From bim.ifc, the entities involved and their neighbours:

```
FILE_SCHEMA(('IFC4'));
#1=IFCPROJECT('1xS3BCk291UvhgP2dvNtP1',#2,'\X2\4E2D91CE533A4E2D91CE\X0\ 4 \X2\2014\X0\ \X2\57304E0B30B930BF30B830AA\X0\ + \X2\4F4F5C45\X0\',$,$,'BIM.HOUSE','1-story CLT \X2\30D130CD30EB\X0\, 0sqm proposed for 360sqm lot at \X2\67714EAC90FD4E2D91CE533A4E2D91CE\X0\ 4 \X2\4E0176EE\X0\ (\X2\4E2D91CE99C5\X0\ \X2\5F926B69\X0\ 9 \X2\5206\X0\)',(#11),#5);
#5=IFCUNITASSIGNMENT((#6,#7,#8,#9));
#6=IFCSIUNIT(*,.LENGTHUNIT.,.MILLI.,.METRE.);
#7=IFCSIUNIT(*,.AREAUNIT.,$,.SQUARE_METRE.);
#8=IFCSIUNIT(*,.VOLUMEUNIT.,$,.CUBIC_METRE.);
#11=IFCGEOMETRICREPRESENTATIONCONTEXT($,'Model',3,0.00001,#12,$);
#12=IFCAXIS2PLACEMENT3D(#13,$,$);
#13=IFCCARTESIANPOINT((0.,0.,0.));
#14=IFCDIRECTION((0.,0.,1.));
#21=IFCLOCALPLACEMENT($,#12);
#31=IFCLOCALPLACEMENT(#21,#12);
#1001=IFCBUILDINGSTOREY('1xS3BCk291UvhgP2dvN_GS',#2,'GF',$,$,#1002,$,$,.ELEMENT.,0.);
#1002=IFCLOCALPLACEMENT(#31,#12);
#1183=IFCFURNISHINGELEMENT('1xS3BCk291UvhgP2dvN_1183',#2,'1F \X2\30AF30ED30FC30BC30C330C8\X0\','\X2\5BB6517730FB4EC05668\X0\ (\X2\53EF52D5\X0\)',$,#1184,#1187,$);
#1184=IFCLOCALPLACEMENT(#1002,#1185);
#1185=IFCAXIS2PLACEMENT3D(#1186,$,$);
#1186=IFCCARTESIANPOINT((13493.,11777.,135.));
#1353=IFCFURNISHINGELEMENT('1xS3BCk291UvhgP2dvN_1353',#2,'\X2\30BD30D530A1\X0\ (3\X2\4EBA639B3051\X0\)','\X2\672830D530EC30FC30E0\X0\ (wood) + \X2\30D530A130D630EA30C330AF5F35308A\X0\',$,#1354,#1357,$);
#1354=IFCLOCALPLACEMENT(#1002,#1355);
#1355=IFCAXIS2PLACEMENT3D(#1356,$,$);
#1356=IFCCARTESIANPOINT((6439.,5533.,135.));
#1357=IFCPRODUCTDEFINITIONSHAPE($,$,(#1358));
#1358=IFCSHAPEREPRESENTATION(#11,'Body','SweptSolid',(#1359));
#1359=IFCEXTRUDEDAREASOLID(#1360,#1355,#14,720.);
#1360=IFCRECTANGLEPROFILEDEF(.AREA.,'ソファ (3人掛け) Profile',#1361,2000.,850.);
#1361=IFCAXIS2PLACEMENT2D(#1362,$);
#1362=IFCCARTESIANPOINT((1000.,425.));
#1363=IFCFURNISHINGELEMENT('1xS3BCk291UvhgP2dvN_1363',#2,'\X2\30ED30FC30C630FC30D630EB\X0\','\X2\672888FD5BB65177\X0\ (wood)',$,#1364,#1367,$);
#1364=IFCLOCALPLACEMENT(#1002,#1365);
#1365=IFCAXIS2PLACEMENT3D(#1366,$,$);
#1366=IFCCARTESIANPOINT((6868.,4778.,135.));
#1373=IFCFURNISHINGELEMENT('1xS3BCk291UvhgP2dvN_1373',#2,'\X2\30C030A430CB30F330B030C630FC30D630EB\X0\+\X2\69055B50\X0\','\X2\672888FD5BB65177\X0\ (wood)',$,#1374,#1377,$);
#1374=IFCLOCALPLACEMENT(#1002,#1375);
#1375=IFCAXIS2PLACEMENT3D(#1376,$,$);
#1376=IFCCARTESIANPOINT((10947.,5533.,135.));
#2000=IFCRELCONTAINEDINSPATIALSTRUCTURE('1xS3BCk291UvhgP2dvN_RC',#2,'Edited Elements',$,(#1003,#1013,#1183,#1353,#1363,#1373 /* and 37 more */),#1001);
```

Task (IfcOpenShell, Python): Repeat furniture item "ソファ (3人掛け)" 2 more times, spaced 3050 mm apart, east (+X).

```python
import numpy as np
import ifcopenshell
import ifcopenshell.api.geometry
import ifcopenshell.api.root
import ifcopenshell.util.element
import ifcopenshell.util.placement
import ifcopenshell.util.unit

model = ifcopenshell.open("bim.ifc")
unit_scale = ifcopenshell.util.unit.calculate_unit_scale(model)


def reuse_history(source, copy):
    """copy_class also copies each property set's owner history, people and application; keep the originals."""
    for rel in copy.IsDefinedBy:
        if rel.is_a("IfcRelDefinesByProperties") and (history := rel.RelatingPropertyDefinition.OwnerHistory):
            rel.RelatingPropertyDefinition.OwnerHistory = source.OwnerHistory
            ifcopenshell.util.element.remove_deep2(model, history)


source = model.by_guid("1xS3BCk291UvhgP2dvN_1353")
base = ifcopenshell.util.placement.get_local_placement(source.ObjectPlacement)
step = np.array([1.0, 0.0, 0.0]) * 3.05 / unit_scale

for i in range(1, 3):
    copy = ifcopenshell.api.root.copy_class(model, product=source)
    copy.Representation = ifcopenshell.util.element.copy_deep(
        model, source.Representation, exclude=["IfcGeometricRepresentationContext", "IfcRepresentationMap"]
    )
    reuse_history(source, copy)
    matrix = base.copy()
    matrix[:3, 3] += i * step
    print("added at", matrix[:3, 3].round(3) + 0.0)
    ifcopenshell.api.geometry.edit_object_placement(model, product=copy, matrix=matrix, is_si=False)

model.write("bim_v2.ifc")
```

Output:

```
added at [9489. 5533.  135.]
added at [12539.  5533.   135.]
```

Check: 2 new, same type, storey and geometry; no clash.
